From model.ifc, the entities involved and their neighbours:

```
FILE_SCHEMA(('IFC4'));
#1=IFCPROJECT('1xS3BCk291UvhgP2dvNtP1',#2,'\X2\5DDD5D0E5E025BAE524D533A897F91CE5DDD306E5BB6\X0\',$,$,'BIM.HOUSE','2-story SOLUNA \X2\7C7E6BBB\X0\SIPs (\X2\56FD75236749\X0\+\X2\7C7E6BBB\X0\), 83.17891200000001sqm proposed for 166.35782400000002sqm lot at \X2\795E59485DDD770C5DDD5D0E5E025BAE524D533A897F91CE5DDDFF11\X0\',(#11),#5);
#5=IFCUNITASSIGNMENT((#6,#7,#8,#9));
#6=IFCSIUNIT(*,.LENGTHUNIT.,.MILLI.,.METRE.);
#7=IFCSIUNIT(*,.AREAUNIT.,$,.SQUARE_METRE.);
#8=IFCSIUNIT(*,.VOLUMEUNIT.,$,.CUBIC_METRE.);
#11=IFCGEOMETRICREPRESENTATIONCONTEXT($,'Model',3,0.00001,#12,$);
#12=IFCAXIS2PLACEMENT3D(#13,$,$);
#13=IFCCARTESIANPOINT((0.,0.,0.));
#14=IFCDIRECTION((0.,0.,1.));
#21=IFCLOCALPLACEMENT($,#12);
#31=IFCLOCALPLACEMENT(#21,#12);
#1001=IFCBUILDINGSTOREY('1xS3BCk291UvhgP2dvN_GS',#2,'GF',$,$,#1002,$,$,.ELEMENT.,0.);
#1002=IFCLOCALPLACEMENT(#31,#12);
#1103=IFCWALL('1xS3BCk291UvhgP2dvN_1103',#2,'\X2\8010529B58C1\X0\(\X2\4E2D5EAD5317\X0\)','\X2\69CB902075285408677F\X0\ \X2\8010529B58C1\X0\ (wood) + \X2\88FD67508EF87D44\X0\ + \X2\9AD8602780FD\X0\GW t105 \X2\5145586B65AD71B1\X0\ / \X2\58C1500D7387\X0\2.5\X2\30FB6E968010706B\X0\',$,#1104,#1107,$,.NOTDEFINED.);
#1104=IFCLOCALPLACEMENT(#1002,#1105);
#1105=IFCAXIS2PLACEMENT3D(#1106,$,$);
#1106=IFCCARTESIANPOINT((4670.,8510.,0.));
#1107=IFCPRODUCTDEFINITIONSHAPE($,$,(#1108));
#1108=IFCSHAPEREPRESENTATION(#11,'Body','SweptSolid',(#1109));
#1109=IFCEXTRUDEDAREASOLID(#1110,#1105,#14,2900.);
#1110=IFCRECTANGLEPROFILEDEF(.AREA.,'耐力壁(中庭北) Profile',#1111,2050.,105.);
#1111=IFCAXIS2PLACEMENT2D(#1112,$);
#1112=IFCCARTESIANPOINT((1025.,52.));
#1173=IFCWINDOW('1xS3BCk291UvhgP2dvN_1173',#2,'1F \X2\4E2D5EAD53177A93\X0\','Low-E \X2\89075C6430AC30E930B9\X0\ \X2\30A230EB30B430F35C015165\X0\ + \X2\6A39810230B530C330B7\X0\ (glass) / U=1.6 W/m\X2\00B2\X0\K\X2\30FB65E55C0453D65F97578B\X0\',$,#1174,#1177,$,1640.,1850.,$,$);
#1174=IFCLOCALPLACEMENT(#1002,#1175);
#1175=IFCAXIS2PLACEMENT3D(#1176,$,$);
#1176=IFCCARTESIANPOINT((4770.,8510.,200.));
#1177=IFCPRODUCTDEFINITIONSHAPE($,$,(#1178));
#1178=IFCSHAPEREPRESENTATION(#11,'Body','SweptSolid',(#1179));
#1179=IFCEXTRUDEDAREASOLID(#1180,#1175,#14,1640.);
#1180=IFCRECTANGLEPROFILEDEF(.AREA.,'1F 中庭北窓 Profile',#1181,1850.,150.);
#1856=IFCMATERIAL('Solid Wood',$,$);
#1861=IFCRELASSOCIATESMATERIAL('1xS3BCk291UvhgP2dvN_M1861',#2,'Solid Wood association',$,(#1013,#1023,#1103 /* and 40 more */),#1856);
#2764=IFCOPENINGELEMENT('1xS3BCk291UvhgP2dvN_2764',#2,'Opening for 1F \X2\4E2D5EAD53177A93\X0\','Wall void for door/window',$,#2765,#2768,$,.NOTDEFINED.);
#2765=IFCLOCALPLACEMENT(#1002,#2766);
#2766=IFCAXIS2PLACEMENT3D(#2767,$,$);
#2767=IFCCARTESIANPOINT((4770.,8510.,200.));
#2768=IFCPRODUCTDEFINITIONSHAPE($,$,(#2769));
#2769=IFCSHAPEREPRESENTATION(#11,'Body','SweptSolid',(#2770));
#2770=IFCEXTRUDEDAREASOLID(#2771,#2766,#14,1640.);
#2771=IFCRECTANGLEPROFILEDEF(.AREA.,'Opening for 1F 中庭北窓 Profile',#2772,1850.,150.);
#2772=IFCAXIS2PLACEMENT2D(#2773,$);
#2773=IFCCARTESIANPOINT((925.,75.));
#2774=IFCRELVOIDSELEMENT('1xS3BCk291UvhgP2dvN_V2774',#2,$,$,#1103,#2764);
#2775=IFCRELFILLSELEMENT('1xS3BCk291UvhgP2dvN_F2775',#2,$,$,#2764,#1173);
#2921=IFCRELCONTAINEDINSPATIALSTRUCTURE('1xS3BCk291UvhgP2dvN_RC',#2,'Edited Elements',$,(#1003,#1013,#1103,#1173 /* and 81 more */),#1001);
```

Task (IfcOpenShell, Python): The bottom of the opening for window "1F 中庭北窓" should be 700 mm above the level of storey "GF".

```python
import numpy as np
import ifcopenshell
import ifcopenshell.api.geometry
import ifcopenshell.geom
import ifcopenshell.util.element
import ifcopenshell.util.placement
import ifcopenshell.util.shape
import ifcopenshell.util.unit

model = ifcopenshell.open("model.ifc")
unit_scale = ifcopenshell.util.unit.calculate_unit_scale(model)

window = model.by_guid("1xS3BCk291UvhgP2dvN_1173")
opening = window.FillsVoids[0].RelatingOpeningElement
storey = ifcopenshell.util.element.get_container(window, ifc_class="IfcBuildingStorey")
level = ifcopenshell.util.placement.get_local_placement(storey.ObjectPlacement)[2, 3]

# The opening's origin need not be at the sill, so measure its lowest point.
shape = ifcopenshell.geom.create_shape(ifcopenshell.geom.settings(), opening)
bottom = ifcopenshell.util.shape.get_shape_bottom_elevation(shape, shape.geometry) / unit_scale
dz = level + 0.7 / unit_scale - bottom

shift = np.array([0.0, 0.0, dz])
# The window is not placed relative to its opening, so move both.
for product in (opening, window):
    matrix = ifcopenshell.util.placement.get_local_placement(product.ObjectPlacement)
    matrix[:3, 3] += shift
    ifcopenshell.api.geometry.edit_object_placement(model, product=product, matrix=matrix, is_si=False)

print(f"moved by {dz * unit_scale:+.3f} m")

model.write("model_edited.ifc")
```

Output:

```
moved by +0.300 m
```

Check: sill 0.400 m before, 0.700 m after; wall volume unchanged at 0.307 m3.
